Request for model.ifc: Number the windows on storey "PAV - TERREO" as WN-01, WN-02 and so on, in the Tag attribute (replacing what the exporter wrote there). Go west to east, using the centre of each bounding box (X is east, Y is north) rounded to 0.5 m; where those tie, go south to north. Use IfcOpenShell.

First a look at what the model holds.

```python
import ifcopenshell
import ifcopenshell.util.element
import ifcopenshell.util.placement

model = ifcopenshell.open("model.ifc")
print(model.schema)
storey = next(s for s in model.by_type("IfcBuildingStorey") if s.Name == "PAV - TERREO")
windows = [e for e in ifcopenshell.util.element.get_decomposition(storey) if e.is_a("IfcWindow")]
for e in sorted(windows, key=lambda e: e.id()):
    origin = ifcopenshell.util.placement.get_local_placement(e.ObjectPlacement)[:3, 3]
    print(e.id(), e.Tag, e.Name, origin.round(2) + 0.0, sep=" | ")
```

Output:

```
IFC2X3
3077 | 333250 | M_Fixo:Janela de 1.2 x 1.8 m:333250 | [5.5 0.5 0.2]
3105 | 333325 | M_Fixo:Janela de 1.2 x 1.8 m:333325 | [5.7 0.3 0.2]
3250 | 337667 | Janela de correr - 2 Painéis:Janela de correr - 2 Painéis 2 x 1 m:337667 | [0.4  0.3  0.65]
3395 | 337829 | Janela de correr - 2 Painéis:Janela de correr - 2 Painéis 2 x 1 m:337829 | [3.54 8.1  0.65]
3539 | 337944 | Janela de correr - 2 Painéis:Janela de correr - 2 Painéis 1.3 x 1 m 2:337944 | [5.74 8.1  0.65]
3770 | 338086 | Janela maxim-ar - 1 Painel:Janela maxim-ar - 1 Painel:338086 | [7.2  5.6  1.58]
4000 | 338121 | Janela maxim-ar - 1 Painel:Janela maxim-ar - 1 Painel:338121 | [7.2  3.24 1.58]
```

```python
import ifcopenshell
import ifcopenshell.geom
import ifcopenshell.util.element
import ifcopenshell.util.shape

model = ifcopenshell.open("model.ifc")
settings = ifcopenshell.geom.settings()
settings.set("use-world-coords", True)


def centre(element):
    shape = ifcopenshell.geom.create_shape(settings, element)
    return ifcopenshell.util.shape.get_bbox_centroid(shape.geometry)


storey = next(s for s in model.by_type("IfcBuildingStorey") if s.Name == "PAV - TERREO")
windows = [e for e in ifcopenshell.util.element.get_decomposition(storey) if e.is_a("IfcWindow")]

# Insertion points can sit at a corner or the storey origin, so sort by the geometry (in metres).
centres = {e: centre(e) for e in windows}
windows.sort(key=lambda e: (round(centres[e][0] / 0.5), centres[e][1]))

for i, e in enumerate(windows, start=1):
    number = f"WN-{i:02d}"
    e.Tag = number
    print(e.id(), number)

model.write("model-out.ifc")
```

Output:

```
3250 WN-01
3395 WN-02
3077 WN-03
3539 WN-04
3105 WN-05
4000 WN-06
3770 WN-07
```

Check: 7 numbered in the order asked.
